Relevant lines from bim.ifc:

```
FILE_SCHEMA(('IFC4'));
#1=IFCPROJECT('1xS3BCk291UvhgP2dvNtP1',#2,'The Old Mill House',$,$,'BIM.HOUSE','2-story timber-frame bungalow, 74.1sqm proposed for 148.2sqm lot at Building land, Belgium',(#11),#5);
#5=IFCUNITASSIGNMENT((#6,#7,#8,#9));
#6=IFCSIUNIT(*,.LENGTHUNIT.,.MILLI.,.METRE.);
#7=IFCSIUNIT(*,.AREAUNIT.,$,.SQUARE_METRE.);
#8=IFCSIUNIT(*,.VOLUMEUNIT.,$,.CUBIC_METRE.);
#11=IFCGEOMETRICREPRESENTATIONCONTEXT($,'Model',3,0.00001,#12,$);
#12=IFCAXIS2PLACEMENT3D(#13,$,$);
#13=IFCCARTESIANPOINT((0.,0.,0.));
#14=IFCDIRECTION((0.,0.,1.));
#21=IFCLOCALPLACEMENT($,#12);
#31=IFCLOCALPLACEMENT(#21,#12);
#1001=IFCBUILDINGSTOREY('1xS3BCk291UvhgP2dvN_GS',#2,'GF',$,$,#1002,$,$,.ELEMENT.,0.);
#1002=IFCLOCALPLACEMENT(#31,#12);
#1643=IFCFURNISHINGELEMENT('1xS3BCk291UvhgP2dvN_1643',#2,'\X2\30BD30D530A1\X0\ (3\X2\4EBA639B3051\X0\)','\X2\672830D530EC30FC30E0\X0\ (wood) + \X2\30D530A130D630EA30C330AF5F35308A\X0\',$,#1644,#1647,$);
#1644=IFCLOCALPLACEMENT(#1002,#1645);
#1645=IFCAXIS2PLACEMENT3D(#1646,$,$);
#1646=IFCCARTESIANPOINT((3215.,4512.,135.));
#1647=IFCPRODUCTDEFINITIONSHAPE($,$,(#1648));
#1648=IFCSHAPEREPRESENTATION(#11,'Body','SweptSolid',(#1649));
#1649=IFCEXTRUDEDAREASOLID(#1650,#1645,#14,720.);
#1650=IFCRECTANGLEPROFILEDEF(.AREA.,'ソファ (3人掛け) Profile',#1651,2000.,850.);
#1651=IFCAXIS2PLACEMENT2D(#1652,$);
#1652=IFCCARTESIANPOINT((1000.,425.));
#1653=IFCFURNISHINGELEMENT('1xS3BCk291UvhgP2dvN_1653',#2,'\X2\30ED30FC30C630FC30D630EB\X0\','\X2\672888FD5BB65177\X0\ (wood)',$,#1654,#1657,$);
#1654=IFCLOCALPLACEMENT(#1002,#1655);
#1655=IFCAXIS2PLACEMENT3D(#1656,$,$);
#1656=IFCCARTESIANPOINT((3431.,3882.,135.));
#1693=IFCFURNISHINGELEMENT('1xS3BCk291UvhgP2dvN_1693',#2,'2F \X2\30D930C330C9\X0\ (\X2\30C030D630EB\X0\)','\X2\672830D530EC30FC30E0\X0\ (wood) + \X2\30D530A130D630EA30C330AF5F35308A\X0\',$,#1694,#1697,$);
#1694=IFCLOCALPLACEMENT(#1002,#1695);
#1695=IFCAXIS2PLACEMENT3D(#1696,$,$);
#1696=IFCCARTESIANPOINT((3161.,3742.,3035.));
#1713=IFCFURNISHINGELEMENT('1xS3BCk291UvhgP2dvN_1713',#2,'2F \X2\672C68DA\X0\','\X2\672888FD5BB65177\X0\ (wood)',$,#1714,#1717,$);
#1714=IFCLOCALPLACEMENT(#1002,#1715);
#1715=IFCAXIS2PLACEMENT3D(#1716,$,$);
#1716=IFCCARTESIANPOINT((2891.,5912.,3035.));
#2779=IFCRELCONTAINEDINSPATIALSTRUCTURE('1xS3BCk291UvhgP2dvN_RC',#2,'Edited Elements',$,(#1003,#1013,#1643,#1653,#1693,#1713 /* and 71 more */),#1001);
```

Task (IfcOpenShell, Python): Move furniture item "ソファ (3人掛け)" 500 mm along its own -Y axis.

```python
import ifcopenshell
import ifcopenshell.api.geometry
import ifcopenshell.util.placement
import ifcopenshell.util.unit

model = ifcopenshell.open("bim.ifc")
unit_scale = ifcopenshell.util.unit.calculate_unit_scale(model)

item = model.by_guid("1xS3BCk291UvhgP2dvN_1643")
matrix = ifcopenshell.util.placement.get_local_placement(item.ObjectPlacement)
matrix[:3, 3] -= matrix[:3, 1] * 0.5 / unit_scale
ifcopenshell.api.geometry.edit_object_placement(model, product=item, matrix=matrix, is_si=False)

print(ifcopenshell.util.placement.get_local_placement(item.ObjectPlacement).round(3) + 0.0)

model.write("bim_rev.ifc")
```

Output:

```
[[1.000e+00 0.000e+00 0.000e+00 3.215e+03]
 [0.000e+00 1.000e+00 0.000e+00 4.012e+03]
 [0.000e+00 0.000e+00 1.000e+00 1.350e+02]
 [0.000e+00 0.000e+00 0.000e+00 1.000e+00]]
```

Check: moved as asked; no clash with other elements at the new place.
